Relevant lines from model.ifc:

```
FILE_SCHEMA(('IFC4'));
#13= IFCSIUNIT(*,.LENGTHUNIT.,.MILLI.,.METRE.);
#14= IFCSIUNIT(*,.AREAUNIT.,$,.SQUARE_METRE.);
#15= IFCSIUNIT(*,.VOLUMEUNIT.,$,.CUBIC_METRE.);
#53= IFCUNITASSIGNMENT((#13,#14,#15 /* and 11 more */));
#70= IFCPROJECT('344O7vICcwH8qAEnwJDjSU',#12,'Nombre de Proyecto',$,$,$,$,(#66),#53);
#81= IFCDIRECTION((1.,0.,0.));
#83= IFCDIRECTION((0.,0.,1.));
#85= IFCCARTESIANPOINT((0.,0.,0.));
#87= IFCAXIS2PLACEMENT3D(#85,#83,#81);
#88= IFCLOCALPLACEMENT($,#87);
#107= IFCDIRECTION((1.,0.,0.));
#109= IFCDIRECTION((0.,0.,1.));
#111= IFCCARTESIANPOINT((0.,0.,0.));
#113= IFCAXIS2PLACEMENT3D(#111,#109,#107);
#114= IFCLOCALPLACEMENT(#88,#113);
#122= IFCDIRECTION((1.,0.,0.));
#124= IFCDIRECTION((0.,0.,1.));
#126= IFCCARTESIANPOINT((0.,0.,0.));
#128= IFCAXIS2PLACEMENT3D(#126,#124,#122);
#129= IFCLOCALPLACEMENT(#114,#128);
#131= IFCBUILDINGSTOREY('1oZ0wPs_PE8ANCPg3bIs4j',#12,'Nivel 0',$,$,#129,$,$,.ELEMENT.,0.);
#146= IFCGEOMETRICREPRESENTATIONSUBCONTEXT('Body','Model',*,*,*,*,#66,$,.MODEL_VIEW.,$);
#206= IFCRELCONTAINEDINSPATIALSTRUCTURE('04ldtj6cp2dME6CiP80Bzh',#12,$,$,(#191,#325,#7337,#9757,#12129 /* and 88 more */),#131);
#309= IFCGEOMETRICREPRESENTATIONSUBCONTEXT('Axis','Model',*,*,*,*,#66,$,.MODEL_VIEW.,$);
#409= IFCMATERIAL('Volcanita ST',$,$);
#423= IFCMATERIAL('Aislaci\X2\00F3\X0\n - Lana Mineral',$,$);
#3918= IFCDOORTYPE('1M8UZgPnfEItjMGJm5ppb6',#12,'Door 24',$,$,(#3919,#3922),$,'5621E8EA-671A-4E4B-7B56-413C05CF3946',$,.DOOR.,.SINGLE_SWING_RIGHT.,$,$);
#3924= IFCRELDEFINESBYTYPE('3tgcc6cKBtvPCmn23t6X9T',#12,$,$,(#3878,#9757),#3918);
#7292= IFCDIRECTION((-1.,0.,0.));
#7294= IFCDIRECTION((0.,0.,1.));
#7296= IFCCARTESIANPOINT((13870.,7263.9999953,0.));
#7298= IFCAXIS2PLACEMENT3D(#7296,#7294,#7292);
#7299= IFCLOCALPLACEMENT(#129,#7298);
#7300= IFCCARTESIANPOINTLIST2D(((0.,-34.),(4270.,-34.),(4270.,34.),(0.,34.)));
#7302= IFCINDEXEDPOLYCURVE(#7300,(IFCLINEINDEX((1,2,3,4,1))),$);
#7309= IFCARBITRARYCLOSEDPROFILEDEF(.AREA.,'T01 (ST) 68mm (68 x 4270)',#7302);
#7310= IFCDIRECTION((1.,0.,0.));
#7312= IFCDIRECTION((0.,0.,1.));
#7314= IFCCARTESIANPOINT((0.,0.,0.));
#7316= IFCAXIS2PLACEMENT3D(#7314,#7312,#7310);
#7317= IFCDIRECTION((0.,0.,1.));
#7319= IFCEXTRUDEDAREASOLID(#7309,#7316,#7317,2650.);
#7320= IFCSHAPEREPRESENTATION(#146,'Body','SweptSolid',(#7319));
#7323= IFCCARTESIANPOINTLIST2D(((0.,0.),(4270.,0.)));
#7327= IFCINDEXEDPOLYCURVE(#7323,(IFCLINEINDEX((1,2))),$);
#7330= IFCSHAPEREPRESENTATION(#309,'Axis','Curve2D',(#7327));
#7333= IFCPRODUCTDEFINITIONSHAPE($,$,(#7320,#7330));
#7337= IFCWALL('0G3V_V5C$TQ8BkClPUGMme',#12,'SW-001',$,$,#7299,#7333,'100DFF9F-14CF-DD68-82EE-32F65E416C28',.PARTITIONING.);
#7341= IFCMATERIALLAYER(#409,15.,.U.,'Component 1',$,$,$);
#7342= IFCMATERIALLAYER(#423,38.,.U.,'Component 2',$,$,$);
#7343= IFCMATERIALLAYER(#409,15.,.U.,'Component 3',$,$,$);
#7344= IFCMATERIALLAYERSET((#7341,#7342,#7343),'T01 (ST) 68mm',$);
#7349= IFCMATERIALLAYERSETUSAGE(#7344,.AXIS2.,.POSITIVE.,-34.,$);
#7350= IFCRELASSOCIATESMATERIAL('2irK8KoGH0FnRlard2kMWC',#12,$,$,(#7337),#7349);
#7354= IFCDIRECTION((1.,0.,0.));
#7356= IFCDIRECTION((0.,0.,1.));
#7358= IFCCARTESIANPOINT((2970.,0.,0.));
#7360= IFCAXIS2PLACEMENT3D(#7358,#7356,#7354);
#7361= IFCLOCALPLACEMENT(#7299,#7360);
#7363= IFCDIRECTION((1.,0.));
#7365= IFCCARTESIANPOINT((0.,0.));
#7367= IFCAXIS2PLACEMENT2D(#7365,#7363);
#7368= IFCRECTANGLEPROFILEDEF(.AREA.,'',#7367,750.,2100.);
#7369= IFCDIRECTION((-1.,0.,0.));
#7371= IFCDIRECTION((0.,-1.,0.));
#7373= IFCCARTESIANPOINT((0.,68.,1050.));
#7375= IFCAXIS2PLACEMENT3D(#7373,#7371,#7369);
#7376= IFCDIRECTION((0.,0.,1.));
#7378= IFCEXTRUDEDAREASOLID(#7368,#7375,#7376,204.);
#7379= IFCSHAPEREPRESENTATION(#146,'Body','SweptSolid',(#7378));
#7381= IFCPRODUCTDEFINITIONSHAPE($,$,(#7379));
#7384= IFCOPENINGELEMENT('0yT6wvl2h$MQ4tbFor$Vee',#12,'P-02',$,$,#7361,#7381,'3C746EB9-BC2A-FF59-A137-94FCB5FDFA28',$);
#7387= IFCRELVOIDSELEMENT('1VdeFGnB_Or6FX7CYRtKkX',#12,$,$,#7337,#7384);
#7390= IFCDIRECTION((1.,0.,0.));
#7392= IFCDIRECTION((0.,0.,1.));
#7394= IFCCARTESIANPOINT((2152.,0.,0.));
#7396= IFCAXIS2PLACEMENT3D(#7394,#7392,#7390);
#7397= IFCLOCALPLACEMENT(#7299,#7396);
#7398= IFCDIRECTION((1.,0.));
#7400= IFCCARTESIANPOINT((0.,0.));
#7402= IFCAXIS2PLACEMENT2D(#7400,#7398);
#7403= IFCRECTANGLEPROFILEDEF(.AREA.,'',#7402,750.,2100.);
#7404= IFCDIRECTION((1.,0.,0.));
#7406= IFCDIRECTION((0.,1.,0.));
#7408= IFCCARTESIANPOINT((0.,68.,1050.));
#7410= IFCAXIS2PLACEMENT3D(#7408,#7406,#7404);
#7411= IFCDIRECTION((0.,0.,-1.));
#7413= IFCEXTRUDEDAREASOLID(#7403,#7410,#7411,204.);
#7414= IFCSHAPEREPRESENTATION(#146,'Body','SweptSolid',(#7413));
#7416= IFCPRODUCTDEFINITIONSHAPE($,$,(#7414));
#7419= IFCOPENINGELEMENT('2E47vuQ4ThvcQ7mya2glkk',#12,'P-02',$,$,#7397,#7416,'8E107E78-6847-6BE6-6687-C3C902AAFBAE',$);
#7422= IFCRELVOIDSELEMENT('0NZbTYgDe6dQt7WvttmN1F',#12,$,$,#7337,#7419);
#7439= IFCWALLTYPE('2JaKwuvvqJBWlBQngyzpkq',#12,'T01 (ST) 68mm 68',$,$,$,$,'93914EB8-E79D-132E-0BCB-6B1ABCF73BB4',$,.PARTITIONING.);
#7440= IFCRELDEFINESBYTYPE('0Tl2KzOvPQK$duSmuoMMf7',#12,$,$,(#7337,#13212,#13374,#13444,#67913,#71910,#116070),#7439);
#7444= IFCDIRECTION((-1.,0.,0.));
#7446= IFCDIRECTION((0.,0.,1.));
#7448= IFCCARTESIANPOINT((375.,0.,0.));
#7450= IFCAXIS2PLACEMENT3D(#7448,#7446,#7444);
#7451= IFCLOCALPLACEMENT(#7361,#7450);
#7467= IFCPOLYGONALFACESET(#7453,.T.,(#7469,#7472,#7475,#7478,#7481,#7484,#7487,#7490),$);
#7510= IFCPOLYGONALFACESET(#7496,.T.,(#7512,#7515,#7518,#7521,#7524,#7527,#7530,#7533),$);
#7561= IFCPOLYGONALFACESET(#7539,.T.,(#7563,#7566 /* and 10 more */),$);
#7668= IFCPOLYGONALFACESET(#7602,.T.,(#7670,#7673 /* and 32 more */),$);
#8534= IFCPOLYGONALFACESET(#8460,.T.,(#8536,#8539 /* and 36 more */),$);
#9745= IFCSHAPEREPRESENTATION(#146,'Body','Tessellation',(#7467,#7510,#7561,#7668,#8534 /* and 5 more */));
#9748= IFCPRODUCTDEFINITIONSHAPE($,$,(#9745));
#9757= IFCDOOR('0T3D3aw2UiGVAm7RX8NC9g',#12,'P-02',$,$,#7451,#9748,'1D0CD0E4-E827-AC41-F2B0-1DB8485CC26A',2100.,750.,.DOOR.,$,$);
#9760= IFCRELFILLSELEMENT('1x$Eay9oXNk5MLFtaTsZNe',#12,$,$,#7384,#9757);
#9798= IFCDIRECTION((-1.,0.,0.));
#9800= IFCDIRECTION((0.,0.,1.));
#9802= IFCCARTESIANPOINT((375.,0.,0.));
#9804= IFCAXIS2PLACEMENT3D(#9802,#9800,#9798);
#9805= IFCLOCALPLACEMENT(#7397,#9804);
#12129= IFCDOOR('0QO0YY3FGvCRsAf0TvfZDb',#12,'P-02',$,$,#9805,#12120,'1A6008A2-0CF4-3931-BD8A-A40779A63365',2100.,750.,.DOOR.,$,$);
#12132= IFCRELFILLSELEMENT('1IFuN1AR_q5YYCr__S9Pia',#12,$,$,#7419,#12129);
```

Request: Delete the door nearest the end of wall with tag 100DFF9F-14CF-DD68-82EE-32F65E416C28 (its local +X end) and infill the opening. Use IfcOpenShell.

```python
import ifcopenshell
import ifcopenshell.api.feature
import ifcopenshell.api.root
import ifcopenshell.geom
import ifcopenshell.util.shape

model = ifcopenshell.open("model.ifc")
settings = ifcopenshell.geom.settings()


def volume(element):
    """Net volume in cubic metres, openings subtracted."""
    shape = ifcopenshell.geom.create_shape(settings, element)
    return ifcopenshell.util.shape.get_volume(shape.geometry)


door = model.by_guid("0T3D3aw2UiGVAm7RX8NC9g")
opening = door.FillsVoids[0].RelatingOpeningElement
wall = opening.VoidsElements[0].RelatingBuildingElement
before = volume(wall)

ifcopenshell.api.root.remove_product(model, product=door)
ifcopenshell.api.feature.remove_feature(model, feature=opening)

after = volume(wall)

print(f"wall volume {before:.3f} -> {after:.3f} m3")

model.write("model_edited.ifc")
```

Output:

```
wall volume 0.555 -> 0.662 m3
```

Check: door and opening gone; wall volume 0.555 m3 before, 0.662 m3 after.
